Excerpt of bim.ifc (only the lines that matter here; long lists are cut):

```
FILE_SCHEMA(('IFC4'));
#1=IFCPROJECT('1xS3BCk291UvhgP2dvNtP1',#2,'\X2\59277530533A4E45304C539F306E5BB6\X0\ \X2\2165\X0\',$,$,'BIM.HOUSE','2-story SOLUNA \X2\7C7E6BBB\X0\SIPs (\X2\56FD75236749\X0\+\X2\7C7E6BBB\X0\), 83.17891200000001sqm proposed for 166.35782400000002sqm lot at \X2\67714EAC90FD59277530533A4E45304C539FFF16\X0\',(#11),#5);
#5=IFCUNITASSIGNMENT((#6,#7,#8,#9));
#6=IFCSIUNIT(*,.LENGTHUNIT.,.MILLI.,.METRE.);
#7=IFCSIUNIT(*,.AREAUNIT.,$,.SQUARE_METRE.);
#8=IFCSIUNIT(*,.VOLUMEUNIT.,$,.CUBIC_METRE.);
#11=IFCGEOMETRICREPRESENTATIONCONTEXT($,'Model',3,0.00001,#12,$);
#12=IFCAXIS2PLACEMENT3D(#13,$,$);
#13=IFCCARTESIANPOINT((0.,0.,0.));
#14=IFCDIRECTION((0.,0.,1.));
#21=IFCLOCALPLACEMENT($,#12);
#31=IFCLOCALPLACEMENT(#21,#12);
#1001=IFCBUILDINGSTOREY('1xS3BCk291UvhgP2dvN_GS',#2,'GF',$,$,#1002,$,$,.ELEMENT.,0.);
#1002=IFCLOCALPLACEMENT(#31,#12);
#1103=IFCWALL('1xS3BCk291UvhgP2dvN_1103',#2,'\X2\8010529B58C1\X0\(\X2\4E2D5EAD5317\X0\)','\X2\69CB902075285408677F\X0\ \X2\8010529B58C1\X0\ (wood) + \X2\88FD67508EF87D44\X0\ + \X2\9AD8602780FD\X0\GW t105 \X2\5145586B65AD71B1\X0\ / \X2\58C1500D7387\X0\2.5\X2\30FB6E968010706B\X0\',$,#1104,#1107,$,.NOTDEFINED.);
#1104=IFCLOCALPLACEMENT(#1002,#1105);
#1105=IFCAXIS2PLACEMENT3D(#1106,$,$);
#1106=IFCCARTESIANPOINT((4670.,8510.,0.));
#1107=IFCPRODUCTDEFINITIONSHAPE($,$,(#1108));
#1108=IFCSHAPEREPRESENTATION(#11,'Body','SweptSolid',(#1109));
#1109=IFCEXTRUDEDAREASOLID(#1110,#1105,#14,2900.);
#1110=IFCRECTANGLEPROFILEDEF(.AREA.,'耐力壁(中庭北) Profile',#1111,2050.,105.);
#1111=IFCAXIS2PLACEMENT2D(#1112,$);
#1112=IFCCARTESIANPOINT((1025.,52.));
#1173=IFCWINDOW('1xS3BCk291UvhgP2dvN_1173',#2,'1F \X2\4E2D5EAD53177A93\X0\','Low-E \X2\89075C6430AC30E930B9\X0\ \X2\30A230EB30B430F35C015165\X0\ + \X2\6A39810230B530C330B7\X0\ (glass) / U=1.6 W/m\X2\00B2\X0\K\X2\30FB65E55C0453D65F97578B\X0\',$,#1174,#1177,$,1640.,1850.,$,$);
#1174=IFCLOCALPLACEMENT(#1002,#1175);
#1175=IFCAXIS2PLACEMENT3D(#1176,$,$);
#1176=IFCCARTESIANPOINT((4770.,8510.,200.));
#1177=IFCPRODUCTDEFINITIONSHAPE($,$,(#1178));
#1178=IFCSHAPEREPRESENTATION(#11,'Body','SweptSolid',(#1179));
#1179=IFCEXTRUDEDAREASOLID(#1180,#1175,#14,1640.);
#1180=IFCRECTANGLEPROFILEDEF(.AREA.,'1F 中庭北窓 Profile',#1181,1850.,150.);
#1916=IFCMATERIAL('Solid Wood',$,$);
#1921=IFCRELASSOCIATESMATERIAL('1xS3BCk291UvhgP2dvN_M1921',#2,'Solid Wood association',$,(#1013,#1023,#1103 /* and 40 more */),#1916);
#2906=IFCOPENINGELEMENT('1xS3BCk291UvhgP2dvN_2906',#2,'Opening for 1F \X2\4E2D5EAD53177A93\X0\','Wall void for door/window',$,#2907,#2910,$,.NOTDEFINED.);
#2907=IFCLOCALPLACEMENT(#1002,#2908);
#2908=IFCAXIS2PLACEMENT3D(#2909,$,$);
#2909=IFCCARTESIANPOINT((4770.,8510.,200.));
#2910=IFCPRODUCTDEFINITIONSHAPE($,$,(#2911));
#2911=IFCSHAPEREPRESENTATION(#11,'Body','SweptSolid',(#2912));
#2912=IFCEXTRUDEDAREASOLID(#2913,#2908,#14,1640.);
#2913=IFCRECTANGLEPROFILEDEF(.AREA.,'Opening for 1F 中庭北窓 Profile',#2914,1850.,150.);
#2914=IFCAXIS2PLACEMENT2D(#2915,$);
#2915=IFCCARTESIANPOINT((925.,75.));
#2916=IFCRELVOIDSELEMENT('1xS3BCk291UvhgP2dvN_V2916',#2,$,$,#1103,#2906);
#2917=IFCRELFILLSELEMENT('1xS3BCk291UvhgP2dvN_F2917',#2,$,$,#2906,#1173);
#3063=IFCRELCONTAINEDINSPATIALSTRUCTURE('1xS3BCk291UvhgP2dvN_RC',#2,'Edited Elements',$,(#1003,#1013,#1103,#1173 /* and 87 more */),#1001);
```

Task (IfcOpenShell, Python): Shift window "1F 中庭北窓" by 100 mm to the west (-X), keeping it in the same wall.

```python
import ifcopenshell
import ifcopenshell.api.geometry
import ifcopenshell.util.placement
import ifcopenshell.util.unit

model = ifcopenshell.open("bim.ifc")
unit_scale = ifcopenshell.util.unit.calculate_unit_scale(model)

window = model.by_guid("1xS3BCk291UvhgP2dvN_1173")
opening = window.FillsVoids[0].RelatingOpeningElement
wall = opening.VoidsElements[0].RelatingBuildingElement

wall_matrix = ifcopenshell.util.placement.get_local_placement(wall.ObjectPlacement)
shift = wall_matrix[:3, 0] * -0.1 / unit_scale
before = ifcopenshell.util.placement.get_local_placement(window.ObjectPlacement)[:3, 3].copy()

# The window is not placed relative to its opening, so move both.
for product in (opening, window):
    matrix = ifcopenshell.util.placement.get_local_placement(product.ObjectPlacement)
    matrix[:3, 3] += shift
    ifcopenshell.api.geometry.edit_object_placement(model, product=product, matrix=matrix, is_si=False)

after = ifcopenshell.util.placement.get_local_placement(window.ObjectPlacement)[:3, 3]
print("window moved by", (after - before).round(3) + 0.0)

model.write("bim_edited.ifc")
```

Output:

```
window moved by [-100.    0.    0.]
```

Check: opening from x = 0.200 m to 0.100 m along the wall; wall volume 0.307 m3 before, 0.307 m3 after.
